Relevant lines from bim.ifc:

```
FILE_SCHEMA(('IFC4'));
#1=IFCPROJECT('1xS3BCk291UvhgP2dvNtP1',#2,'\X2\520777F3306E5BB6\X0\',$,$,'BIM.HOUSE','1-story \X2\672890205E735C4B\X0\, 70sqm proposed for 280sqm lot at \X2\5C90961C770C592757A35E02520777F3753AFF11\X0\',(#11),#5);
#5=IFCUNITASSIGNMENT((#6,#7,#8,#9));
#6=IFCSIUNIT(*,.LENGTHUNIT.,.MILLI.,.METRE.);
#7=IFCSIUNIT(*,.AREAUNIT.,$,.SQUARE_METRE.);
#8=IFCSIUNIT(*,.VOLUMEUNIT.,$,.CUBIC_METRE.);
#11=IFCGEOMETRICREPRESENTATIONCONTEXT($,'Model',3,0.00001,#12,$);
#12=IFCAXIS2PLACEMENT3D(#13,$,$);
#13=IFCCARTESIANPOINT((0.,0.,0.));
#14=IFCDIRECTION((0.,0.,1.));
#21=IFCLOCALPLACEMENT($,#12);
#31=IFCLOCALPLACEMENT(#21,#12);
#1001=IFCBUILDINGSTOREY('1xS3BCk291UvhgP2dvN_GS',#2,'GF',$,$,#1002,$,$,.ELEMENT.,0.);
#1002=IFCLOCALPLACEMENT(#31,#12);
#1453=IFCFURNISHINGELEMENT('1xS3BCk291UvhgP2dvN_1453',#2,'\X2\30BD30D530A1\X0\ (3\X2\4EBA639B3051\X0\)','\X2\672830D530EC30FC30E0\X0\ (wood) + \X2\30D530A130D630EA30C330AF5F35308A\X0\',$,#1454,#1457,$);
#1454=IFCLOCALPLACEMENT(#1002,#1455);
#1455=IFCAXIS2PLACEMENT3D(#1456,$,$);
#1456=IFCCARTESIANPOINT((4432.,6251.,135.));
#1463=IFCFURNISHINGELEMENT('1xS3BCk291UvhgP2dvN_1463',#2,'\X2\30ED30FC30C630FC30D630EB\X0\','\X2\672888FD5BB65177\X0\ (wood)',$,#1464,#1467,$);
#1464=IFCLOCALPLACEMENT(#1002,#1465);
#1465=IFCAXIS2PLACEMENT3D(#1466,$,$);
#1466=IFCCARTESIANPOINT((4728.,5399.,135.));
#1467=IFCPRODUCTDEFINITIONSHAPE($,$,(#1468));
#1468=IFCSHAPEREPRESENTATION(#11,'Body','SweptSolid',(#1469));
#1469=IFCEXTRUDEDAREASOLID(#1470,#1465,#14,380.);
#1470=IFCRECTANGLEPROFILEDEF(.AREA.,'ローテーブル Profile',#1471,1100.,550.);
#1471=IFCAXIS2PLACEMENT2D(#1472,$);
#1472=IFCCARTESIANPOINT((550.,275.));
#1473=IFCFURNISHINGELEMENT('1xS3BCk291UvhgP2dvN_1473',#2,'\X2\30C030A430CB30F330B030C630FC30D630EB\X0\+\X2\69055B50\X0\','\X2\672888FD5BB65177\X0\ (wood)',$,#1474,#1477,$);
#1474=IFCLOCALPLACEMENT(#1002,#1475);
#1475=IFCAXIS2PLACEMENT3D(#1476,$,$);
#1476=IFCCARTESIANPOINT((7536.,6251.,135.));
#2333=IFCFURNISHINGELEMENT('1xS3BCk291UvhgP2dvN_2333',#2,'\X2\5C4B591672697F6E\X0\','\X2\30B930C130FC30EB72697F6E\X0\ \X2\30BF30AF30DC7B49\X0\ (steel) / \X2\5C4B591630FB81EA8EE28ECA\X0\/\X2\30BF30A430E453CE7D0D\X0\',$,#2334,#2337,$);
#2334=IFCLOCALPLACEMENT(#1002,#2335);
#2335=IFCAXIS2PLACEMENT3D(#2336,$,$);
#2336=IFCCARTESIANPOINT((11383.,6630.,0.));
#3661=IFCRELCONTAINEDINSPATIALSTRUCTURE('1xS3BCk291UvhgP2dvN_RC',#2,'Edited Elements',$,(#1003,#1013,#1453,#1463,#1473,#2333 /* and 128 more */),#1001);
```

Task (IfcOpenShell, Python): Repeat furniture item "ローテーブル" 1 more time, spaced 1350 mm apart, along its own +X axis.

```python
import ifcopenshell
import ifcopenshell.api.geometry
import ifcopenshell.api.root
import ifcopenshell.util.element
import ifcopenshell.util.placement

model = ifcopenshell.open("bim.ifc")


def reuse_history(source, copy):
    """copy_class also copies each property set's owner history, people and application; keep the originals."""
    for rel in copy.IsDefinedBy:
        if rel.is_a("IfcRelDefinesByProperties") and (history := rel.RelatingPropertyDefinition.OwnerHistory):
            rel.RelatingPropertyDefinition.OwnerHistory = source.OwnerHistory
            ifcopenshell.util.element.remove_deep2(model, history)


source = model.by_guid("1xS3BCk291UvhgP2dvN_1463")
base = ifcopenshell.util.placement.get_local_placement(source.ObjectPlacement)
step = base[:3, 0] * 1350.0

for i in range(1, 2):
    copy = ifcopenshell.api.root.copy_class(model, product=source)
    copy.Representation = ifcopenshell.util.element.copy_deep(
        model, source.Representation, exclude=["IfcGeometricRepresentationContext", "IfcRepresentationMap"]
    )
    reuse_history(source, copy)
    matrix = base.copy()
    matrix[:3, 3] += i * step
    print("added at", matrix[:3, 3].round(3) + 0.0)
    ifcopenshell.api.geometry.edit_object_placement(model, product=copy, matrix=matrix, is_si=False)

model.write("bim-out.ifc")
```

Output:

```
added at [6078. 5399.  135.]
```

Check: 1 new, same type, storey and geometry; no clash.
